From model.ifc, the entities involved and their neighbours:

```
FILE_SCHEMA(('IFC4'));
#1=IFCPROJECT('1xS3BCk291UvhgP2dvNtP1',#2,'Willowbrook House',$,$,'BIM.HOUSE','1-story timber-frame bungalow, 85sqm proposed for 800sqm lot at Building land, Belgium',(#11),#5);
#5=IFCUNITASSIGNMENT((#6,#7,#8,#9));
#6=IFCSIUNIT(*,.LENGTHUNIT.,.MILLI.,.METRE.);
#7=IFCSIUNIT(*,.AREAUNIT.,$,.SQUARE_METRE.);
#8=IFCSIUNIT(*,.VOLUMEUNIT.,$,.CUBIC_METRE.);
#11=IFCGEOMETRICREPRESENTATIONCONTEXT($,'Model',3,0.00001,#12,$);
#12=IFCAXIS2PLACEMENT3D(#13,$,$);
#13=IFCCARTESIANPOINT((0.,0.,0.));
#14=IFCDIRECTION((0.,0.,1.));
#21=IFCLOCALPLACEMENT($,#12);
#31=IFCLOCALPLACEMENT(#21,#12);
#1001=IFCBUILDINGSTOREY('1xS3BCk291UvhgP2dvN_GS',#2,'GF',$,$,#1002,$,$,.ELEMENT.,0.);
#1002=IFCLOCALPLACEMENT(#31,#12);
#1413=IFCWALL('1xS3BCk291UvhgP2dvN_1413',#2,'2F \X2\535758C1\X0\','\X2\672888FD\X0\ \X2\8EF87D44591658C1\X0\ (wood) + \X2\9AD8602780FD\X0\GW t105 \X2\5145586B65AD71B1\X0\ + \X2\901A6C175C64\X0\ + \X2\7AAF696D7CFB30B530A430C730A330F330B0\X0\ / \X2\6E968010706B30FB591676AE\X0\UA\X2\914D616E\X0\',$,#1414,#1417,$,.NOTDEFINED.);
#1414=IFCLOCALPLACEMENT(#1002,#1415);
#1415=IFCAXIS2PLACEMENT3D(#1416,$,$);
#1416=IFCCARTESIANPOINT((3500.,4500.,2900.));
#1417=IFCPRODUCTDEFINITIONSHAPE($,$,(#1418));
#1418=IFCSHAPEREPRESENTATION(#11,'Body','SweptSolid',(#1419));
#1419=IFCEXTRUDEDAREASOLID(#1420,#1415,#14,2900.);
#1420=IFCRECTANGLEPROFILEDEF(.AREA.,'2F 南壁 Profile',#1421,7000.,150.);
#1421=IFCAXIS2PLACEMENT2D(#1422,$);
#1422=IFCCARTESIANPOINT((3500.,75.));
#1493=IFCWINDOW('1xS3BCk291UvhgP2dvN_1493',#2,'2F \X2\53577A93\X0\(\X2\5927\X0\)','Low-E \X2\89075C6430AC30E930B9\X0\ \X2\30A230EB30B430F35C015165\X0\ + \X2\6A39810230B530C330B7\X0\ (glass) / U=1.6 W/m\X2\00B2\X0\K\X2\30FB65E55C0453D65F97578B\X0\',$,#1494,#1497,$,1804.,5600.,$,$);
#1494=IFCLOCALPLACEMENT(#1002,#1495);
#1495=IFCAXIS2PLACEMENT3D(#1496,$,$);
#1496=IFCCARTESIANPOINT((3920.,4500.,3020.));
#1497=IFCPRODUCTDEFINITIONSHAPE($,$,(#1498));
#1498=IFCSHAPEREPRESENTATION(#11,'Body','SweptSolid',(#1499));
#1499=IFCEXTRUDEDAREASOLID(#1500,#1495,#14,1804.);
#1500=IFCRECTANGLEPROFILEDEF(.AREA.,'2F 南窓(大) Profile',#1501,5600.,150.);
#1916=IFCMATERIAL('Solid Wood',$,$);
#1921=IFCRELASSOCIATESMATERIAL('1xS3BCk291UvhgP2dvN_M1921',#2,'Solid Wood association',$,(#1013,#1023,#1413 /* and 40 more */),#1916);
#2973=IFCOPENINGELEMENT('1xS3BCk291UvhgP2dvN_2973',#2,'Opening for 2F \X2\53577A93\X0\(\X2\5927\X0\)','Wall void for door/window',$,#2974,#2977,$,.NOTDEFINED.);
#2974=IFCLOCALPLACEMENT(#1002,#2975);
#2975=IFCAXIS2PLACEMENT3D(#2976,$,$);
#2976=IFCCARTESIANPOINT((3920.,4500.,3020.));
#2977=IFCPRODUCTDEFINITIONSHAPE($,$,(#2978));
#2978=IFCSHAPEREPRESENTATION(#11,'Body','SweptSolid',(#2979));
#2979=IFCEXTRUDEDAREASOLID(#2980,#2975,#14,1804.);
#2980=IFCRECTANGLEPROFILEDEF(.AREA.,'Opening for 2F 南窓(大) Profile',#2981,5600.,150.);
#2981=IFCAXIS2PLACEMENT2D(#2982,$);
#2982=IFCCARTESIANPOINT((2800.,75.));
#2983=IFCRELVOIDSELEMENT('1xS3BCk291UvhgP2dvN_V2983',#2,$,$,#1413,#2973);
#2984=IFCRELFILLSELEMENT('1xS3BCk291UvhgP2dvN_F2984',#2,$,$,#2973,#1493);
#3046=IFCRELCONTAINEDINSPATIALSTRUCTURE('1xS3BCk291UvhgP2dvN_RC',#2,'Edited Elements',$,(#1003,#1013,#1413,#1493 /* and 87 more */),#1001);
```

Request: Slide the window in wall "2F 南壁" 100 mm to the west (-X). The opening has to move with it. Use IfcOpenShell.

```python
import ifcopenshell
import ifcopenshell.api.geometry
import ifcopenshell.util.placement
import ifcopenshell.util.unit

model = ifcopenshell.open("model.ifc")
unit_scale = ifcopenshell.util.unit.calculate_unit_scale(model)

window = model.by_guid("1xS3BCk291UvhgP2dvN_1493")
opening = window.FillsVoids[0].RelatingOpeningElement
wall = opening.VoidsElements[0].RelatingBuildingElement

wall_matrix = ifcopenshell.util.placement.get_local_placement(wall.ObjectPlacement)
shift = wall_matrix[:3, 0] * -0.1 / unit_scale
before = ifcopenshell.util.placement.get_local_placement(window.ObjectPlacement)[:3, 3].copy()

# The window is not placed relative to its opening, so move both.
for product in (opening, window):
    matrix = ifcopenshell.util.placement.get_local_placement(product.ObjectPlacement)
    matrix[:3, 3] += shift
    ifcopenshell.api.geometry.edit_object_placement(model, product=product, matrix=matrix, is_si=False)

after = ifcopenshell.util.placement.get_local_placement(window.ObjectPlacement)[:3, 3]
print("window moved by", (after - before).round(3) + 0.0)

model.write("model_v2.ifc")
```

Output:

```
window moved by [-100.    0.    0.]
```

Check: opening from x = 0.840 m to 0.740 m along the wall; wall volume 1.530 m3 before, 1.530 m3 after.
